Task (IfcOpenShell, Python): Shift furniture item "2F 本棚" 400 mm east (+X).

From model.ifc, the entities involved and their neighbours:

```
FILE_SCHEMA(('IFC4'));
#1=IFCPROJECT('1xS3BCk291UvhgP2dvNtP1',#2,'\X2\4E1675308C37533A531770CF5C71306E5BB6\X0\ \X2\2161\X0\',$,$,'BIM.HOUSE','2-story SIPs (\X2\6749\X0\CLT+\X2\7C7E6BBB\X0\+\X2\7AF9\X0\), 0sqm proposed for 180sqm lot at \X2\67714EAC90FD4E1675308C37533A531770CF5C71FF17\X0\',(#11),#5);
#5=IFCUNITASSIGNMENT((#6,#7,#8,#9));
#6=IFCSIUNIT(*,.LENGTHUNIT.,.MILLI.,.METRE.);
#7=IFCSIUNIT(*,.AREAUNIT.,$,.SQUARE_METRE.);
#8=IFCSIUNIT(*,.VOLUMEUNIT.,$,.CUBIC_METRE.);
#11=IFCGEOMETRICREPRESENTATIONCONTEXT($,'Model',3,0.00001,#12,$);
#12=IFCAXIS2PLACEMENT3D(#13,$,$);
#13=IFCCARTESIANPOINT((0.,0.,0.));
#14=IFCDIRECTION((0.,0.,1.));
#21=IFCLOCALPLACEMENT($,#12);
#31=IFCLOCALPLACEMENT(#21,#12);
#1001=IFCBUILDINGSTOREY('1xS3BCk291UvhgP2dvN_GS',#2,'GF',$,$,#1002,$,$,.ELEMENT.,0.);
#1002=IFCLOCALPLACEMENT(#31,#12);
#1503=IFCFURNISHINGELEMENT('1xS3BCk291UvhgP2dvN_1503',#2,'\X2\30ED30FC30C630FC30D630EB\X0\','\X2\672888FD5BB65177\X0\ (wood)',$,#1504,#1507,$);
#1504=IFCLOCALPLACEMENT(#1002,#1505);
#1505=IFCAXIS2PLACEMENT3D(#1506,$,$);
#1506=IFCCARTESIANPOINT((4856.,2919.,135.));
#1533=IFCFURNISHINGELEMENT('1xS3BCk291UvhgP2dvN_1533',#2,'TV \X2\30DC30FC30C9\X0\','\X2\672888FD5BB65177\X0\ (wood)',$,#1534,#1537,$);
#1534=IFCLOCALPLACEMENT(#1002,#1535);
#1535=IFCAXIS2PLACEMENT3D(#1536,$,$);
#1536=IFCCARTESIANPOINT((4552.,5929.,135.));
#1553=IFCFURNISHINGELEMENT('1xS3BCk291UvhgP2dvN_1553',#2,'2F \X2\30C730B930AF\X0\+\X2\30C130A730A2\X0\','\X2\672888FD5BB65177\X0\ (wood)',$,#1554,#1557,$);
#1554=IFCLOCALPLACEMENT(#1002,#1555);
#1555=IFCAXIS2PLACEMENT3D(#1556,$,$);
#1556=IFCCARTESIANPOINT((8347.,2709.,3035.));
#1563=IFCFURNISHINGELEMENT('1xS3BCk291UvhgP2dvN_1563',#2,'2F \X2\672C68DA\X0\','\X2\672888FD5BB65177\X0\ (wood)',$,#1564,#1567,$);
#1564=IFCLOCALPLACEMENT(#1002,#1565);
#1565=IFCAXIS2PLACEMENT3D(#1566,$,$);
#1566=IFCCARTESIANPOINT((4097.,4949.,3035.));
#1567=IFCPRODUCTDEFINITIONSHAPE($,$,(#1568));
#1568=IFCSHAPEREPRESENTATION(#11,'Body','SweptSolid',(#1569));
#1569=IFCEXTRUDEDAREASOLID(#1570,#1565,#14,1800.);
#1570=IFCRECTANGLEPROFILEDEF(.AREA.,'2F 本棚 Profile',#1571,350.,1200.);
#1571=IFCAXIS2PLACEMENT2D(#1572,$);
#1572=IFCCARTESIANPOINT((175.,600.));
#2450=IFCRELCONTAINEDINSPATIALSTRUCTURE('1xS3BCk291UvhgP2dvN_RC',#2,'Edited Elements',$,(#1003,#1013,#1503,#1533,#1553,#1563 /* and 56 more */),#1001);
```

```python
import ifcopenshell
import ifcopenshell.api.geometry
import ifcopenshell.util.placement
import ifcopenshell.util.unit

model = ifcopenshell.open("model.ifc")
unit_scale = ifcopenshell.util.unit.calculate_unit_scale(model)

item = model.by_guid("1xS3BCk291UvhgP2dvN_1563")
matrix = ifcopenshell.util.placement.get_local_placement(item.ObjectPlacement)
matrix[0, 3] += 0.4 / unit_scale
ifcopenshell.api.geometry.edit_object_placement(model, product=item, matrix=matrix, is_si=False)

print(ifcopenshell.util.placement.get_local_placement(item.ObjectPlacement).round(3) + 0.0)

model.write("model_rev.ifc")
```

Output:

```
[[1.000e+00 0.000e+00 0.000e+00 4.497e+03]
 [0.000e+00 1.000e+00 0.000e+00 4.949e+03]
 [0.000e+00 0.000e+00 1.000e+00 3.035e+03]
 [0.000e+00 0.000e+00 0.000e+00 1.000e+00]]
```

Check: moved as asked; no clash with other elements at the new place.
